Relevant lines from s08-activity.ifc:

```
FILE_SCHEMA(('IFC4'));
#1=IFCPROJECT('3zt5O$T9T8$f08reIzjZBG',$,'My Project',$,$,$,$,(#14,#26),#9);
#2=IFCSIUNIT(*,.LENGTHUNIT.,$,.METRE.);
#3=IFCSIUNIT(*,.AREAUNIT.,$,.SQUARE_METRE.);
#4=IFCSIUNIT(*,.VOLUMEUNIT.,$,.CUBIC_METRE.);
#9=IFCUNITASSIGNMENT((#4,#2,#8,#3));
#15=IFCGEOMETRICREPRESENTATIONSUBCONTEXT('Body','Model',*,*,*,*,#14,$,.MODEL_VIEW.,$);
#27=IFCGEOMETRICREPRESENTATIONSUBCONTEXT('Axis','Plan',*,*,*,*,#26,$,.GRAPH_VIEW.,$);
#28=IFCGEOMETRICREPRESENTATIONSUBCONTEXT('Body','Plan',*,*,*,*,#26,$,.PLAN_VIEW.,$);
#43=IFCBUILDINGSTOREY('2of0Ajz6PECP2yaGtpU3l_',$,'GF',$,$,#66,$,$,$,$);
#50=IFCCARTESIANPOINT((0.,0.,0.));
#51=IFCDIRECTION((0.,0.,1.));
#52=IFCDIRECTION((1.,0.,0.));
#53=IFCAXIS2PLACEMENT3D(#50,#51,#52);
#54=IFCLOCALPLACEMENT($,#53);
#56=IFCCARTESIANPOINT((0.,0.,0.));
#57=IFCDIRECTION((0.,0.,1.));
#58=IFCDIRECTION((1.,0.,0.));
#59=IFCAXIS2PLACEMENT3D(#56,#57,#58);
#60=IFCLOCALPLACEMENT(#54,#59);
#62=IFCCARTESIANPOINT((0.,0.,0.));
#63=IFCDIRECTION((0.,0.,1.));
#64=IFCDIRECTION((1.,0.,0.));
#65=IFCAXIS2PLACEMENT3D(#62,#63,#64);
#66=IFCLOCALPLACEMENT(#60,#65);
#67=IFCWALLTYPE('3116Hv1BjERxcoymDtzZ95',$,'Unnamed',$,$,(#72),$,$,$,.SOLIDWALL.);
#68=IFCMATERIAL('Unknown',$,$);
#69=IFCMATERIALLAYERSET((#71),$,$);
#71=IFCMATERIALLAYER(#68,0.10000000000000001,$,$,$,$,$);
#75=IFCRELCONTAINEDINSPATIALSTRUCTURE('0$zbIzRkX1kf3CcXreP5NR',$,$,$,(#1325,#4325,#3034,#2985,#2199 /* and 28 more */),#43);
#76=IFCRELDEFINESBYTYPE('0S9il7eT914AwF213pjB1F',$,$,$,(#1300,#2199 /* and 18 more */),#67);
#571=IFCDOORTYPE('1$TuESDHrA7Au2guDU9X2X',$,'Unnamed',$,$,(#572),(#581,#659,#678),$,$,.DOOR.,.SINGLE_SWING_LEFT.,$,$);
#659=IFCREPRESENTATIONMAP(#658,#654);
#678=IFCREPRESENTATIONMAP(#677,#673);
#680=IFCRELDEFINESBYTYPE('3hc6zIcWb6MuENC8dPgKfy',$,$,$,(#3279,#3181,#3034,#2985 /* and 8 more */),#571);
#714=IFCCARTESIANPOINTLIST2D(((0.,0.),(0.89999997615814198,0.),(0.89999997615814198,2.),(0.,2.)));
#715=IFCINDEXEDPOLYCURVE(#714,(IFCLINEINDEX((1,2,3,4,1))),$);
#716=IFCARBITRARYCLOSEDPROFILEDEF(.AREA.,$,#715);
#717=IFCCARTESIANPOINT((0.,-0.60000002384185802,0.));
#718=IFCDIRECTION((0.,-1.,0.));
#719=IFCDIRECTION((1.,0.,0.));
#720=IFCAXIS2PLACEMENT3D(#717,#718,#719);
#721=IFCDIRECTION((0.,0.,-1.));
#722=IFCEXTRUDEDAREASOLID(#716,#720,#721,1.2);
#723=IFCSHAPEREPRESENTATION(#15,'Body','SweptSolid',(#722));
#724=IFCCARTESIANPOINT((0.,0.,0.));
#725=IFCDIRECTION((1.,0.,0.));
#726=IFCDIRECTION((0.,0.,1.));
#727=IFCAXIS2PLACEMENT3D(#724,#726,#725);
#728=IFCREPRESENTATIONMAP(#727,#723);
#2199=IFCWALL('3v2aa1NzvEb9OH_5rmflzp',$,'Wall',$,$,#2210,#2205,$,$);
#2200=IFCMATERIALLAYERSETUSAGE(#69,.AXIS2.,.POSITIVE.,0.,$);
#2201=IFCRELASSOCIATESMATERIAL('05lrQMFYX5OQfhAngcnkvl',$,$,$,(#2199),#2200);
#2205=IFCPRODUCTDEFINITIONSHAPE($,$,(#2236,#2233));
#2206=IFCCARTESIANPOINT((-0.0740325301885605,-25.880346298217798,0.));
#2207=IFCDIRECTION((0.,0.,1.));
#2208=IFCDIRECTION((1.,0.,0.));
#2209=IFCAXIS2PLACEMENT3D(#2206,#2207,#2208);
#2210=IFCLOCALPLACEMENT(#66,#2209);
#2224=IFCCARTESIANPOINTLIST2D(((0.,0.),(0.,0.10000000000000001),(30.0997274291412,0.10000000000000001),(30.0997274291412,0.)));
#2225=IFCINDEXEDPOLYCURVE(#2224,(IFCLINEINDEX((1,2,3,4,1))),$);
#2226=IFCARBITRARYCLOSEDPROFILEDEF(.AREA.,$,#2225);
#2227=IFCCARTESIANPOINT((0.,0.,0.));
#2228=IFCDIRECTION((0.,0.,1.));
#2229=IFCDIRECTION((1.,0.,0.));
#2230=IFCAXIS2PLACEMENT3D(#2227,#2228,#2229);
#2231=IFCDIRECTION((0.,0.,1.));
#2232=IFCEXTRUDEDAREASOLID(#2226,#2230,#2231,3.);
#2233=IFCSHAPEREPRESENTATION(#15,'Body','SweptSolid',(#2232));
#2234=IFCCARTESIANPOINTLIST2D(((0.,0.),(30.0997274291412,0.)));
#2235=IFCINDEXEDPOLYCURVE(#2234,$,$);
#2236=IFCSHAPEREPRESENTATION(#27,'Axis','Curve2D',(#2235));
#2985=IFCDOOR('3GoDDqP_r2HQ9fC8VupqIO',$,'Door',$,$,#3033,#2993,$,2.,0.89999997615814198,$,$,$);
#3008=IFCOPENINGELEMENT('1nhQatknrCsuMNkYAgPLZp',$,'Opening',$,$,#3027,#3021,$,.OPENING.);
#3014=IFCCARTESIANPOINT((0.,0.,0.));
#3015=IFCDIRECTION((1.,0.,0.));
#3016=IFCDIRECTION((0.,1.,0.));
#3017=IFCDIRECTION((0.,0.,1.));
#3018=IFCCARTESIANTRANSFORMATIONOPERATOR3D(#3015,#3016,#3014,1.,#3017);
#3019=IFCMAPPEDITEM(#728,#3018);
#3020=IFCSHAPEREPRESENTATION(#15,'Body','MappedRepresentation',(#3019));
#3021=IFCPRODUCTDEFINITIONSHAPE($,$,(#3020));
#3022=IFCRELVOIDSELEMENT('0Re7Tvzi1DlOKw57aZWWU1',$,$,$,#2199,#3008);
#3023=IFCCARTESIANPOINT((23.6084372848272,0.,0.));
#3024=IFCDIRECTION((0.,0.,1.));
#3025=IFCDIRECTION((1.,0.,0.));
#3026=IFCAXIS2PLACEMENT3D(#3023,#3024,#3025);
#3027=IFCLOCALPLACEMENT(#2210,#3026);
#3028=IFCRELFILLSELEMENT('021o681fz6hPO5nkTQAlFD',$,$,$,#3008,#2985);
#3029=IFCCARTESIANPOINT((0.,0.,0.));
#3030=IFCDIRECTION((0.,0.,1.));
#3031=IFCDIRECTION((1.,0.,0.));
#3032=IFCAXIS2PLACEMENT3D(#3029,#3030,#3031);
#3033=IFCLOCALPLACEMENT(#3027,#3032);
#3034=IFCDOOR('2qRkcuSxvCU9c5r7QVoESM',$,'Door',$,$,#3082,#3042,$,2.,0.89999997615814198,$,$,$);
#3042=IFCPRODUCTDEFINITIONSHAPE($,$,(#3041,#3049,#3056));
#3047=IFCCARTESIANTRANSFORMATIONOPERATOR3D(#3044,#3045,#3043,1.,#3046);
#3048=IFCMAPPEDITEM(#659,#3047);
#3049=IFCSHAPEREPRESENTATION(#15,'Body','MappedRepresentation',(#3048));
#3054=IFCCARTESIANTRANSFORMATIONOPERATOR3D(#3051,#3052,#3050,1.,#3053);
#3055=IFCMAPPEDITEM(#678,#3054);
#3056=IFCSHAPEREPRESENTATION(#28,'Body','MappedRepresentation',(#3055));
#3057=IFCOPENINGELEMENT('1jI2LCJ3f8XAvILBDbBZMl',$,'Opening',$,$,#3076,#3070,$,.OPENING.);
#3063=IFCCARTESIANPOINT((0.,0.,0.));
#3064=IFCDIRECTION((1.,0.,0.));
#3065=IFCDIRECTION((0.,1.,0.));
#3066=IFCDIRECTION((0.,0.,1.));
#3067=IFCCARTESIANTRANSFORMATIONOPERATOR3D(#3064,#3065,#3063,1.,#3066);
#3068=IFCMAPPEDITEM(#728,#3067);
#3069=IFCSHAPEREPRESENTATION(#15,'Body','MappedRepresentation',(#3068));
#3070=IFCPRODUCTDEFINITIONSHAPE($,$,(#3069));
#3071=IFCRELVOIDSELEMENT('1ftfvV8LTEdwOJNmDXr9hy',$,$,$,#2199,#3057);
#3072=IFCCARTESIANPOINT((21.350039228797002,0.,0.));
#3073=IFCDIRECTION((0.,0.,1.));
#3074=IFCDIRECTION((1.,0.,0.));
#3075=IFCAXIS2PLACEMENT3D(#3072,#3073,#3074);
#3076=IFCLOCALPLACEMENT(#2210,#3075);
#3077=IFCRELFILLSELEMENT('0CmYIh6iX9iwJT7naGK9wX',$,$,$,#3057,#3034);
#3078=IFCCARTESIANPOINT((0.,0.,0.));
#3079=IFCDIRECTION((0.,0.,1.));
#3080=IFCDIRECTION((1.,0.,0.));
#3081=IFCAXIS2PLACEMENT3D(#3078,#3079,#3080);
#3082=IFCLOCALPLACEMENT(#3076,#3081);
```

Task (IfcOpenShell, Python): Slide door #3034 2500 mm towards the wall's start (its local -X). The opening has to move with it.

```python
import ifcopenshell
import ifcopenshell.api.geometry
import ifcopenshell.util.placement
import ifcopenshell.util.unit

model = ifcopenshell.open("s08-activity.ifc")
unit_scale = ifcopenshell.util.unit.calculate_unit_scale(model)

door = model.by_guid("2qRkcuSxvCU9c5r7QVoESM")
opening = door.FillsVoids[0].RelatingOpeningElement
wall = opening.VoidsElements[0].RelatingBuildingElement

wall_matrix = ifcopenshell.util.placement.get_local_placement(wall.ObjectPlacement)
shift = wall_matrix[:3, 0] * -2.5 / unit_scale
before = ifcopenshell.util.placement.get_local_placement(door.ObjectPlacement)[:3, 3].copy()

# The door is placed relative to its opening, so it follows when the opening moves.
matrix = ifcopenshell.util.placement.get_local_placement(opening.ObjectPlacement)
matrix[:3, 3] += shift
ifcopenshell.api.geometry.edit_object_placement(
    model, product=opening, matrix=matrix, is_si=False, should_transform_children=True
)

after = ifcopenshell.util.placement.get_local_placement(door.ObjectPlacement)[:3, 3]
print("door moved by", (after - before).round(3) + 0.0)

model.write("s08-activity_v2.ifc")
```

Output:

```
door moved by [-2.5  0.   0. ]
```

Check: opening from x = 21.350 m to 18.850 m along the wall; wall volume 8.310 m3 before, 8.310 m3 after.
